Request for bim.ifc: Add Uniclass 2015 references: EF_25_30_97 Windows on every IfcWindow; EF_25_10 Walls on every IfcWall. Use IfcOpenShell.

First a look at what the model holds.

```python
import ifcopenshell

model = ifcopenshell.open("bim.ifc")
print(model.schema)
print("classifications:", [c.Name for c in model.by_type("IfcClassification")])
for ifc_class in ("IfcDoor", "IfcRoof", "IfcStair", "IfcWall", "IfcWindow"):
    print(ifc_class, len(model.by_type(ifc_class)))
```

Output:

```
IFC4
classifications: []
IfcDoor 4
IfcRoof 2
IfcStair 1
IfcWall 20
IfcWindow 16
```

```python
import ifcopenshell
import ifcopenshell.api.classification

model = ifcopenshell.open("bim.ifc")

system = ifcopenshell.api.classification.add_classification(model, classification="Uniclass 2015")

codes = {
    "IfcWindow": ("EF_25_30_97", "Windows"),
    "IfcWall": ("EF_25_10", "Walls"),
}
for ifc_class, (code, name) in codes.items():
    products = model.by_type(ifc_class)
    ifcopenshell.api.classification.add_reference(
        model, products=products, classification=system, identification=code, name=name
    )
    print(code, len(products))

model.write("bim_v2.ifc")
```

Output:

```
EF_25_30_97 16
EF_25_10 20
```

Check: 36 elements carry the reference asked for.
